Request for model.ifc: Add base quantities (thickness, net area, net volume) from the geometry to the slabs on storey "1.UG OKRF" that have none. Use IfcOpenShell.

First a look at what the model holds.

```python
import ifcopenshell
import ifcopenshell.util.element
import ifcopenshell.util.unit

model = ifcopenshell.open("model.ifc")
print(model.schema)
for unit_type in ("LENGTHUNIT", "AREAUNIT", "VOLUMEUNIT"):
    print(unit_type, ifcopenshell.util.unit.calculate_unit_scale(model, unit_type))
storey = next(s for s in model.by_type("IfcBuildingStorey") if s.Name == "1.UG OKRF")
slabs = [e for e in ifcopenshell.util.element.get_decomposition(storey) if e.is_a("IfcSlab")]
for e in sorted(slabs, key=lambda e: e.id()):
    print(e.id(), e.is_a(), e.Name, list(ifcopenshell.util.element.get_psets(e, qtos_only=True)), sep=" | ")
```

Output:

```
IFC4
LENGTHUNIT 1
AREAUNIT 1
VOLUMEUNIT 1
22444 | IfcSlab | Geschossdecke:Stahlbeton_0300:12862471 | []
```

```python
import ifcopenshell
import ifcopenshell.api.pset
import ifcopenshell.geom
import ifcopenshell.util.element
import ifcopenshell.util.shape
import ifcopenshell.util.unit

model = ifcopenshell.open("model.ifc")
unit_scale = ifcopenshell.util.unit.calculate_unit_scale(model)
area_scale = ifcopenshell.util.unit.calculate_unit_scale(model, "AREAUNIT")
volume_scale = ifcopenshell.util.unit.calculate_unit_scale(model, "VOLUMEUNIT")
settings = ifcopenshell.geom.settings()

storey = next(s for s in model.by_type("IfcBuildingStorey") if s.Name == "1.UG OKRF")
slabs = [e for e in ifcopenshell.util.element.get_decomposition(storey) if e.is_a("IfcSlab")]

for e in sorted(slabs, key=lambda e: e.id()):
    if ifcopenshell.util.element.get_psets(e, qtos_only=True, should_inherit=False):
        continue
    # Geometry comes back in metres, in the element's own axes.
    shape = ifcopenshell.geom.create_shape(settings, e)
    values = {
        "Width": ifcopenshell.util.shape.get_z(shape.geometry) / unit_scale,
        "NetArea": ifcopenshell.util.shape.get_footprint_area(shape.geometry) / area_scale,
        "NetVolume": ifcopenshell.util.shape.get_volume(shape.geometry) / volume_scale,
    }
    qto = ifcopenshell.api.pset.add_qto(model, product=e, name="Qto_SlabBaseQuantities")
    ifcopenshell.api.pset.edit_qto(model, qto=qto, properties=values)
    print(e.id(), {k: round(v, 3) for k, v in values.items()})

model.write("model_updated.ifc")
```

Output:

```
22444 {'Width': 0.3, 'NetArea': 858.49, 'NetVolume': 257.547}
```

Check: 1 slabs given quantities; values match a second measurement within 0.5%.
